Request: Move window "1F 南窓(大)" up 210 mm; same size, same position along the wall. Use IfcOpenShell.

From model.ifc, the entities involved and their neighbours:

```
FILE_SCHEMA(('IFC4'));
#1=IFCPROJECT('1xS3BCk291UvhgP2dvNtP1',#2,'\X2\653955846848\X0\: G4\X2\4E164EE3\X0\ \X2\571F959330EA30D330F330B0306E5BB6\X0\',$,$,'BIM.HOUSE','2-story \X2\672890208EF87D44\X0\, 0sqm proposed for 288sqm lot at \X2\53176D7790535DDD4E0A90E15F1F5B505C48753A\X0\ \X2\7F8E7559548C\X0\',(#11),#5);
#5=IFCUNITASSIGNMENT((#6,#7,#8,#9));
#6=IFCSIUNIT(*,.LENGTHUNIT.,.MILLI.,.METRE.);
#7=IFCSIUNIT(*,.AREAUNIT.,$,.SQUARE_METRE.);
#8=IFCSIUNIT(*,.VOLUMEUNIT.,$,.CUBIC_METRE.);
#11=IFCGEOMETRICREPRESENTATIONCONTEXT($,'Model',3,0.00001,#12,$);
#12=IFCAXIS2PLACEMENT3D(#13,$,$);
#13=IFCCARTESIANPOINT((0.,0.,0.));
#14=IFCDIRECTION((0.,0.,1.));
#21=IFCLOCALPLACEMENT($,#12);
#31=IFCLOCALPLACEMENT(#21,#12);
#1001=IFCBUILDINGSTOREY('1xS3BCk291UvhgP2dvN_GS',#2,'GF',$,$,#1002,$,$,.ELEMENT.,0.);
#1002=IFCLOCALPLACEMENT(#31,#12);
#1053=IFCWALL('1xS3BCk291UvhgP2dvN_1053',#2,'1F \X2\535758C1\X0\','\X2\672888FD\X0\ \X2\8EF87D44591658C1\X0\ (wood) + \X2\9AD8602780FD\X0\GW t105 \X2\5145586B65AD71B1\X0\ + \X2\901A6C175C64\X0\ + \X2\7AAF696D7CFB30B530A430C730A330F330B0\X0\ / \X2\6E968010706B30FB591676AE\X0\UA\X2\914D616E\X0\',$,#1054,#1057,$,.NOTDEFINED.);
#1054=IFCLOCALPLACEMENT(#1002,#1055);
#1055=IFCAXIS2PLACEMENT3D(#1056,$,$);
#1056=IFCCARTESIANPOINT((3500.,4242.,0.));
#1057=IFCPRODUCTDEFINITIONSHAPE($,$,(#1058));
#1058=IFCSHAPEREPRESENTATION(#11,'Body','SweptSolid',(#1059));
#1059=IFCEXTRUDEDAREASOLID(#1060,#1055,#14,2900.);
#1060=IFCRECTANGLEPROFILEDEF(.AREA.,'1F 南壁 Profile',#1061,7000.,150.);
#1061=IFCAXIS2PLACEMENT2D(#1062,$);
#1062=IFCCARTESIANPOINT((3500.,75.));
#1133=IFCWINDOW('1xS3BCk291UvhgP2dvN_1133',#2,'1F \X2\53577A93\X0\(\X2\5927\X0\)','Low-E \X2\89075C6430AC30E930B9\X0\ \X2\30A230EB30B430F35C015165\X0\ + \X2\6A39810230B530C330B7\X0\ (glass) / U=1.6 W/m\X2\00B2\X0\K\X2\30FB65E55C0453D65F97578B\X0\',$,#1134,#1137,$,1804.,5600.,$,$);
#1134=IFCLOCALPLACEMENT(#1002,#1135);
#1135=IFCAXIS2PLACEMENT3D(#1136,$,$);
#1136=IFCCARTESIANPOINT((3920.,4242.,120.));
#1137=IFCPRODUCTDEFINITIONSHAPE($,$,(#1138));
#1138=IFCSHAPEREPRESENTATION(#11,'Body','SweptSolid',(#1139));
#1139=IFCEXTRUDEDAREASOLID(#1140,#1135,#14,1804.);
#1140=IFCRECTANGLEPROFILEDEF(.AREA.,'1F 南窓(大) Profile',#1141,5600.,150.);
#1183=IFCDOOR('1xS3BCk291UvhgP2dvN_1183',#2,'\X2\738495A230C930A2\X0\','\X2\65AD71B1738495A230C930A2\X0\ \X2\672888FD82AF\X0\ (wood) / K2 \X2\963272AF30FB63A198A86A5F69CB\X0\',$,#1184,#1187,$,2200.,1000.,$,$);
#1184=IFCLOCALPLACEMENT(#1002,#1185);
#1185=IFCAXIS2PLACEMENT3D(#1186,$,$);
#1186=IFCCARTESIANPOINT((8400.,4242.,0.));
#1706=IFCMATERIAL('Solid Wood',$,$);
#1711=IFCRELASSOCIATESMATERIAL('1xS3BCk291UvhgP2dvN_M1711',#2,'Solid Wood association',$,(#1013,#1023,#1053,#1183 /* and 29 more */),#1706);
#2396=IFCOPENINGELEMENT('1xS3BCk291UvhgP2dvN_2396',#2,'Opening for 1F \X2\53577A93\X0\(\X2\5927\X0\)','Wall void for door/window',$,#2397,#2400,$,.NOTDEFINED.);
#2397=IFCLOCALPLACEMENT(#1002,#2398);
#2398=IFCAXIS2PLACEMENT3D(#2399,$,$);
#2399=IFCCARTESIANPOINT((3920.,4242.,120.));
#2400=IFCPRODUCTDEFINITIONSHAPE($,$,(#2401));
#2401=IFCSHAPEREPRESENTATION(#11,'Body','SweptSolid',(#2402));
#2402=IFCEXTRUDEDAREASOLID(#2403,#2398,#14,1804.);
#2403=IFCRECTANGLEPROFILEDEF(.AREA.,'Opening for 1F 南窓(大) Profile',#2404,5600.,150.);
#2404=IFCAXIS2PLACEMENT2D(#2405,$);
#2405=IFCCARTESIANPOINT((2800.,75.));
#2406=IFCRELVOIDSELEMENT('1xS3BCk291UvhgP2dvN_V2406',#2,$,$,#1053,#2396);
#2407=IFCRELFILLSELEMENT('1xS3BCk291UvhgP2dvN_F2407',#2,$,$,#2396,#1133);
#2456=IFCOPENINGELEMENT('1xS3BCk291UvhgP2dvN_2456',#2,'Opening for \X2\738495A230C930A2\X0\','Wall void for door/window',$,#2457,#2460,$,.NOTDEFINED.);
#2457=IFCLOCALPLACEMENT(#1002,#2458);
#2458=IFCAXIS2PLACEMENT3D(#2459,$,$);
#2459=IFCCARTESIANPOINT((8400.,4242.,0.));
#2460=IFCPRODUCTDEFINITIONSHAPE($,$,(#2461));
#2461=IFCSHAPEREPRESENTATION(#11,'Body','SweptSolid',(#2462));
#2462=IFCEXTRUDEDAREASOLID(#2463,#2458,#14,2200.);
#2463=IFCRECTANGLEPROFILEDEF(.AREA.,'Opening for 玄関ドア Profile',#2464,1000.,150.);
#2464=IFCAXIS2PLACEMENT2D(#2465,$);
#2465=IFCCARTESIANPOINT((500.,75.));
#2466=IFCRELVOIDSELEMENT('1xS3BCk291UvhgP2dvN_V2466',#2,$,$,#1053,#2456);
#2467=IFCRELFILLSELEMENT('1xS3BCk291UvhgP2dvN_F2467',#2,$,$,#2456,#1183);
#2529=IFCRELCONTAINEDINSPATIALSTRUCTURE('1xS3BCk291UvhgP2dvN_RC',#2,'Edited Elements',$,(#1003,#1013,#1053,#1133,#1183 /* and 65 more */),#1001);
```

```python
import numpy as np
import ifcopenshell
import ifcopenshell.api.geometry
import ifcopenshell.util.placement
import ifcopenshell.util.unit

model = ifcopenshell.open("model.ifc")
unit_scale = ifcopenshell.util.unit.calculate_unit_scale(model)

window = model.by_guid("1xS3BCk291UvhgP2dvN_1133")
opening = window.FillsVoids[0].RelatingOpeningElement
dz = 210.0

shift = np.array([0.0, 0.0, dz])
# The window is not placed relative to its opening, so move both.
for product in (opening, window):
    matrix = ifcopenshell.util.placement.get_local_placement(product.ObjectPlacement)
    matrix[:3, 3] += shift
    ifcopenshell.api.geometry.edit_object_placement(model, product=product, matrix=matrix, is_si=False)

print(f"moved by {dz * unit_scale:+.3f} m")

model.write("model_edited.ifc")
```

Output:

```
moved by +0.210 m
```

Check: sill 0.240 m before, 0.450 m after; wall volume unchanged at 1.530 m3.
